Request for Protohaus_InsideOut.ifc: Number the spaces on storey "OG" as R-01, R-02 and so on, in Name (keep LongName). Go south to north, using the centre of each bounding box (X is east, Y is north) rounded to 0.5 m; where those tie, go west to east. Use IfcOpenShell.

First a look at what the model holds.

```python
import ifcopenshell
import ifcopenshell.util.element
import ifcopenshell.util.placement

model = ifcopenshell.open("Protohaus_InsideOut.ifc")
print(model.schema)
storey = next(s for s in model.by_type("IfcBuildingStorey") if s.Name == "OG")
spaces = [e for e in ifcopenshell.util.element.get_decomposition(storey) if e.is_a("IfcSpace")]
for e in sorted(spaces, key=lambda e: e.id()):
    origin = ifcopenshell.util.placement.get_local_placement(e.ObjectPlacement)[:3, 3]
    print(e.id(), e.Name, e.LongName, origin.round(2) + 0.0, sep=" | ")
```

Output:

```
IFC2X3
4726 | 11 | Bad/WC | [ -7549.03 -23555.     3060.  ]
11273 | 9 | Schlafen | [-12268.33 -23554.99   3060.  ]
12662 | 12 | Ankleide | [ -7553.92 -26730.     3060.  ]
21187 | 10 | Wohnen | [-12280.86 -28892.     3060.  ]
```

```python
import ifcopenshell
import ifcopenshell.geom
import ifcopenshell.util.element
import ifcopenshell.util.shape

model = ifcopenshell.open("Protohaus_InsideOut.ifc")
settings = ifcopenshell.geom.settings()
settings.set("use-world-coords", True)


def centre(element):
    shape = ifcopenshell.geom.create_shape(settings, element)
    return ifcopenshell.util.shape.get_bbox_centroid(shape.geometry)


storey = next(s for s in model.by_type("IfcBuildingStorey") if s.Name == "OG")
spaces = [e for e in ifcopenshell.util.element.get_decomposition(storey) if e.is_a("IfcSpace")]

# Insertion points can sit at a corner or the storey origin, so sort by the geometry (in metres).
centres = {e: centre(e) for e in spaces}
spaces.sort(key=lambda e: (round(centres[e][1] / 0.5), centres[e][0]))

for i, e in enumerate(spaces, start=1):
    number = f"R-{i:02d}"
    e.Name = number
    print(e.id(), number)

model.write("Protohaus_InsideOut_updated.ifc")
```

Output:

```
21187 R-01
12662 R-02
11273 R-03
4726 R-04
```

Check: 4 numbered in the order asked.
